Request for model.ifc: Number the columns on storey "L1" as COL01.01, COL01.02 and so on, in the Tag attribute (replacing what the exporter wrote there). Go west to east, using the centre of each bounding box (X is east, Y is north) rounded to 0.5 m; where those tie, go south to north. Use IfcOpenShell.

First a look at what the model holds.

```python
import ifcopenshell
import ifcopenshell.util.element
import ifcopenshell.util.placement

model = ifcopenshell.open("model.ifc")
print(model.schema)
storey = next(s for s in model.by_type("IfcBuildingStorey") if s.Name == "L1")
columns = [e for e in ifcopenshell.util.element.get_decomposition(storey) if e.is_a("IfcColumn")]
for e in sorted(columns, key=lambda e: e.id()):
    origin = ifcopenshell.util.placement.get_local_placement(e.ObjectPlacement)[:3, 3]
    print(e.id(), e.Tag, e.Name, origin.round(2) + 0.0, sep=" | ")
```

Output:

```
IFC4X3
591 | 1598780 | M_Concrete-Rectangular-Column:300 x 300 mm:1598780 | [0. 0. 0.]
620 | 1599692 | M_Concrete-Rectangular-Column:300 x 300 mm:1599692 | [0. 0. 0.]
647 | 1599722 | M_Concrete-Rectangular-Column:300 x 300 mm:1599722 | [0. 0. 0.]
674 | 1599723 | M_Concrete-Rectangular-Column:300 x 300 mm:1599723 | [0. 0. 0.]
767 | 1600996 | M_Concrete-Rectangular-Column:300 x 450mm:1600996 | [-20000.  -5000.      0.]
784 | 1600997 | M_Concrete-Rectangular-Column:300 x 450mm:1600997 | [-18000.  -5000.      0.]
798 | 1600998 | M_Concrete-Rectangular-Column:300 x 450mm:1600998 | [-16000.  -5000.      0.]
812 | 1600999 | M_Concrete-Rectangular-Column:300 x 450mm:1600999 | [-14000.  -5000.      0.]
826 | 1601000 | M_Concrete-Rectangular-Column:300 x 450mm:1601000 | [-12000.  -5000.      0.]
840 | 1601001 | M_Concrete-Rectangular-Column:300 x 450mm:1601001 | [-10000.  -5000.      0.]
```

```python
import ifcopenshell
import ifcopenshell.geom
import ifcopenshell.util.element
import ifcopenshell.util.shape

model = ifcopenshell.open("model.ifc")
settings = ifcopenshell.geom.settings()
settings.set("use-world-coords", True)


def centre(element):
    shape = ifcopenshell.geom.create_shape(settings, element)
    return ifcopenshell.util.shape.get_bbox_centroid(shape.geometry)


storey = next(s for s in model.by_type("IfcBuildingStorey") if s.Name == "L1")
columns = [e for e in ifcopenshell.util.element.get_decomposition(storey) if e.is_a("IfcColumn")]

# Insertion points can sit at a corner or the storey origin, so sort by the geometry (in metres).
centres = {e: centre(e) for e in columns}
columns.sort(key=lambda e: (round(centres[e][0] / 0.5), centres[e][1]))

for i, e in enumerate(columns, start=1):
    number = f"COL01.{i:02d}"
    e.Tag = number
    print(e.id(), number)

model.write("model_rev.ifc")
```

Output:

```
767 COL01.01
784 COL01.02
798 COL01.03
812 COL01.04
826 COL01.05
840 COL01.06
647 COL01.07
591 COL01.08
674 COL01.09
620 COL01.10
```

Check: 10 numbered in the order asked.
